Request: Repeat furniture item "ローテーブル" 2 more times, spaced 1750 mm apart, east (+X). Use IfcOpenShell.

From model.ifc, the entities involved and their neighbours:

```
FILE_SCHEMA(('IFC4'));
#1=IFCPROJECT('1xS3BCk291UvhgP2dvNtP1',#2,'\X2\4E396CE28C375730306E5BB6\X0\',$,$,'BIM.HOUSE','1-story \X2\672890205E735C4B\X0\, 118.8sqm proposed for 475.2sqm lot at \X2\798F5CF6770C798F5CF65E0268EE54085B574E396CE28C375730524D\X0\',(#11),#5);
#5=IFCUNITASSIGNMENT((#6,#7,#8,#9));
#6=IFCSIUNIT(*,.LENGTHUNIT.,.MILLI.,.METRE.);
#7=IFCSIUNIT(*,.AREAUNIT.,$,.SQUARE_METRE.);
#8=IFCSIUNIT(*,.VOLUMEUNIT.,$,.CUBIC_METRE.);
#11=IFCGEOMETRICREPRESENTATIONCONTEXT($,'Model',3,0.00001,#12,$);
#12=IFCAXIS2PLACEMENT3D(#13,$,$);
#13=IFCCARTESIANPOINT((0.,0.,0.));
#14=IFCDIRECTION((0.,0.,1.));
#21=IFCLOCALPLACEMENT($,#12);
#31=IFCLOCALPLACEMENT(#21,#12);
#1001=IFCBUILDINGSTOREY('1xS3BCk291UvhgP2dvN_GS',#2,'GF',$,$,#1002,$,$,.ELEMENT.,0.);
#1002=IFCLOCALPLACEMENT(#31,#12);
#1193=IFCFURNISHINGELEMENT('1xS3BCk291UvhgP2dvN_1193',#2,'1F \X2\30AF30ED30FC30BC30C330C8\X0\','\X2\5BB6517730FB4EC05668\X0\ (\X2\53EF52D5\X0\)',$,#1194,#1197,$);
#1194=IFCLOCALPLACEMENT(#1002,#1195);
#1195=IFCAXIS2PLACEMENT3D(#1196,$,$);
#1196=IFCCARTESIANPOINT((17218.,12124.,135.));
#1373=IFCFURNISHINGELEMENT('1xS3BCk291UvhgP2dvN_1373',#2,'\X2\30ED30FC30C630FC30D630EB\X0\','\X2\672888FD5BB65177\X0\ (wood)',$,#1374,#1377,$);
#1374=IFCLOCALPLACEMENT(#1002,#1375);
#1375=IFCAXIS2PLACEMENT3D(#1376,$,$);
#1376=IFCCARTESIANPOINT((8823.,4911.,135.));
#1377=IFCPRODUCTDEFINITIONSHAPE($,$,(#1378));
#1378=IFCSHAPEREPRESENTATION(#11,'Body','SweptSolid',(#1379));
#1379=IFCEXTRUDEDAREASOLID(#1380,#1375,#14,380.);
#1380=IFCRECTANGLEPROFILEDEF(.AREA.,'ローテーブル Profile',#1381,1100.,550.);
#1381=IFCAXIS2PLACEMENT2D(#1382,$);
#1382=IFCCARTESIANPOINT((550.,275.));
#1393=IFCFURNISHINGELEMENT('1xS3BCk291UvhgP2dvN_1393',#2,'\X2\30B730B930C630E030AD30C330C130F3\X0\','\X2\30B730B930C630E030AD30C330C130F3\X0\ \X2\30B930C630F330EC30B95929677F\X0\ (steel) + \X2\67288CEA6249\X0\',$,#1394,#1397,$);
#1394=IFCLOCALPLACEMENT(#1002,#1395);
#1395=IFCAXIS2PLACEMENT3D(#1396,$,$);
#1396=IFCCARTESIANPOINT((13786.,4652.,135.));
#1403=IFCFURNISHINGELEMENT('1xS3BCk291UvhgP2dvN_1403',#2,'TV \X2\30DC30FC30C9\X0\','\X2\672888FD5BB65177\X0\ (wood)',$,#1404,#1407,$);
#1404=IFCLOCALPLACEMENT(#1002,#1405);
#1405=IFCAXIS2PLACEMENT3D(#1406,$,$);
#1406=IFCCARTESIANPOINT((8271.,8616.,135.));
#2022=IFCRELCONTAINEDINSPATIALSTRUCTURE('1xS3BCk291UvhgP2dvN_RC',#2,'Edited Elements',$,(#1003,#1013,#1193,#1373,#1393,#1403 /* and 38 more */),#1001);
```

```python
import numpy as np
import ifcopenshell
import ifcopenshell.api.geometry
import ifcopenshell.api.root
import ifcopenshell.util.element
import ifcopenshell.util.placement
import ifcopenshell.util.unit

model = ifcopenshell.open("model.ifc")
unit_scale = ifcopenshell.util.unit.calculate_unit_scale(model)


def reuse_history(source, copy):
    """copy_class also copies each property set's owner history, people and application; keep the originals."""
    for rel in copy.IsDefinedBy:
        if rel.is_a("IfcRelDefinesByProperties") and (history := rel.RelatingPropertyDefinition.OwnerHistory):
            rel.RelatingPropertyDefinition.OwnerHistory = source.OwnerHistory
            ifcopenshell.util.element.remove_deep2(model, history)


source = model.by_guid("1xS3BCk291UvhgP2dvN_1373")
base = ifcopenshell.util.placement.get_local_placement(source.ObjectPlacement)
step = np.array([1.0, 0.0, 0.0]) * 1.75 / unit_scale

for i in range(1, 3):
    copy = ifcopenshell.api.root.copy_class(model, product=source)
    copy.Representation = ifcopenshell.util.element.copy_deep(
        model, source.Representation, exclude=["IfcGeometricRepresentationContext", "IfcRepresentationMap"]
    )
    reuse_history(source, copy)
    matrix = base.copy()
    matrix[:3, 3] += i * step
    print("added at", matrix[:3, 3].round(3) + 0.0)
    ifcopenshell.api.geometry.edit_object_placement(model, product=copy, matrix=matrix, is_si=False)

model.write("model_updated.ifc")
```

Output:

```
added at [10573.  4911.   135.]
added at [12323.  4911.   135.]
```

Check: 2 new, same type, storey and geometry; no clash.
